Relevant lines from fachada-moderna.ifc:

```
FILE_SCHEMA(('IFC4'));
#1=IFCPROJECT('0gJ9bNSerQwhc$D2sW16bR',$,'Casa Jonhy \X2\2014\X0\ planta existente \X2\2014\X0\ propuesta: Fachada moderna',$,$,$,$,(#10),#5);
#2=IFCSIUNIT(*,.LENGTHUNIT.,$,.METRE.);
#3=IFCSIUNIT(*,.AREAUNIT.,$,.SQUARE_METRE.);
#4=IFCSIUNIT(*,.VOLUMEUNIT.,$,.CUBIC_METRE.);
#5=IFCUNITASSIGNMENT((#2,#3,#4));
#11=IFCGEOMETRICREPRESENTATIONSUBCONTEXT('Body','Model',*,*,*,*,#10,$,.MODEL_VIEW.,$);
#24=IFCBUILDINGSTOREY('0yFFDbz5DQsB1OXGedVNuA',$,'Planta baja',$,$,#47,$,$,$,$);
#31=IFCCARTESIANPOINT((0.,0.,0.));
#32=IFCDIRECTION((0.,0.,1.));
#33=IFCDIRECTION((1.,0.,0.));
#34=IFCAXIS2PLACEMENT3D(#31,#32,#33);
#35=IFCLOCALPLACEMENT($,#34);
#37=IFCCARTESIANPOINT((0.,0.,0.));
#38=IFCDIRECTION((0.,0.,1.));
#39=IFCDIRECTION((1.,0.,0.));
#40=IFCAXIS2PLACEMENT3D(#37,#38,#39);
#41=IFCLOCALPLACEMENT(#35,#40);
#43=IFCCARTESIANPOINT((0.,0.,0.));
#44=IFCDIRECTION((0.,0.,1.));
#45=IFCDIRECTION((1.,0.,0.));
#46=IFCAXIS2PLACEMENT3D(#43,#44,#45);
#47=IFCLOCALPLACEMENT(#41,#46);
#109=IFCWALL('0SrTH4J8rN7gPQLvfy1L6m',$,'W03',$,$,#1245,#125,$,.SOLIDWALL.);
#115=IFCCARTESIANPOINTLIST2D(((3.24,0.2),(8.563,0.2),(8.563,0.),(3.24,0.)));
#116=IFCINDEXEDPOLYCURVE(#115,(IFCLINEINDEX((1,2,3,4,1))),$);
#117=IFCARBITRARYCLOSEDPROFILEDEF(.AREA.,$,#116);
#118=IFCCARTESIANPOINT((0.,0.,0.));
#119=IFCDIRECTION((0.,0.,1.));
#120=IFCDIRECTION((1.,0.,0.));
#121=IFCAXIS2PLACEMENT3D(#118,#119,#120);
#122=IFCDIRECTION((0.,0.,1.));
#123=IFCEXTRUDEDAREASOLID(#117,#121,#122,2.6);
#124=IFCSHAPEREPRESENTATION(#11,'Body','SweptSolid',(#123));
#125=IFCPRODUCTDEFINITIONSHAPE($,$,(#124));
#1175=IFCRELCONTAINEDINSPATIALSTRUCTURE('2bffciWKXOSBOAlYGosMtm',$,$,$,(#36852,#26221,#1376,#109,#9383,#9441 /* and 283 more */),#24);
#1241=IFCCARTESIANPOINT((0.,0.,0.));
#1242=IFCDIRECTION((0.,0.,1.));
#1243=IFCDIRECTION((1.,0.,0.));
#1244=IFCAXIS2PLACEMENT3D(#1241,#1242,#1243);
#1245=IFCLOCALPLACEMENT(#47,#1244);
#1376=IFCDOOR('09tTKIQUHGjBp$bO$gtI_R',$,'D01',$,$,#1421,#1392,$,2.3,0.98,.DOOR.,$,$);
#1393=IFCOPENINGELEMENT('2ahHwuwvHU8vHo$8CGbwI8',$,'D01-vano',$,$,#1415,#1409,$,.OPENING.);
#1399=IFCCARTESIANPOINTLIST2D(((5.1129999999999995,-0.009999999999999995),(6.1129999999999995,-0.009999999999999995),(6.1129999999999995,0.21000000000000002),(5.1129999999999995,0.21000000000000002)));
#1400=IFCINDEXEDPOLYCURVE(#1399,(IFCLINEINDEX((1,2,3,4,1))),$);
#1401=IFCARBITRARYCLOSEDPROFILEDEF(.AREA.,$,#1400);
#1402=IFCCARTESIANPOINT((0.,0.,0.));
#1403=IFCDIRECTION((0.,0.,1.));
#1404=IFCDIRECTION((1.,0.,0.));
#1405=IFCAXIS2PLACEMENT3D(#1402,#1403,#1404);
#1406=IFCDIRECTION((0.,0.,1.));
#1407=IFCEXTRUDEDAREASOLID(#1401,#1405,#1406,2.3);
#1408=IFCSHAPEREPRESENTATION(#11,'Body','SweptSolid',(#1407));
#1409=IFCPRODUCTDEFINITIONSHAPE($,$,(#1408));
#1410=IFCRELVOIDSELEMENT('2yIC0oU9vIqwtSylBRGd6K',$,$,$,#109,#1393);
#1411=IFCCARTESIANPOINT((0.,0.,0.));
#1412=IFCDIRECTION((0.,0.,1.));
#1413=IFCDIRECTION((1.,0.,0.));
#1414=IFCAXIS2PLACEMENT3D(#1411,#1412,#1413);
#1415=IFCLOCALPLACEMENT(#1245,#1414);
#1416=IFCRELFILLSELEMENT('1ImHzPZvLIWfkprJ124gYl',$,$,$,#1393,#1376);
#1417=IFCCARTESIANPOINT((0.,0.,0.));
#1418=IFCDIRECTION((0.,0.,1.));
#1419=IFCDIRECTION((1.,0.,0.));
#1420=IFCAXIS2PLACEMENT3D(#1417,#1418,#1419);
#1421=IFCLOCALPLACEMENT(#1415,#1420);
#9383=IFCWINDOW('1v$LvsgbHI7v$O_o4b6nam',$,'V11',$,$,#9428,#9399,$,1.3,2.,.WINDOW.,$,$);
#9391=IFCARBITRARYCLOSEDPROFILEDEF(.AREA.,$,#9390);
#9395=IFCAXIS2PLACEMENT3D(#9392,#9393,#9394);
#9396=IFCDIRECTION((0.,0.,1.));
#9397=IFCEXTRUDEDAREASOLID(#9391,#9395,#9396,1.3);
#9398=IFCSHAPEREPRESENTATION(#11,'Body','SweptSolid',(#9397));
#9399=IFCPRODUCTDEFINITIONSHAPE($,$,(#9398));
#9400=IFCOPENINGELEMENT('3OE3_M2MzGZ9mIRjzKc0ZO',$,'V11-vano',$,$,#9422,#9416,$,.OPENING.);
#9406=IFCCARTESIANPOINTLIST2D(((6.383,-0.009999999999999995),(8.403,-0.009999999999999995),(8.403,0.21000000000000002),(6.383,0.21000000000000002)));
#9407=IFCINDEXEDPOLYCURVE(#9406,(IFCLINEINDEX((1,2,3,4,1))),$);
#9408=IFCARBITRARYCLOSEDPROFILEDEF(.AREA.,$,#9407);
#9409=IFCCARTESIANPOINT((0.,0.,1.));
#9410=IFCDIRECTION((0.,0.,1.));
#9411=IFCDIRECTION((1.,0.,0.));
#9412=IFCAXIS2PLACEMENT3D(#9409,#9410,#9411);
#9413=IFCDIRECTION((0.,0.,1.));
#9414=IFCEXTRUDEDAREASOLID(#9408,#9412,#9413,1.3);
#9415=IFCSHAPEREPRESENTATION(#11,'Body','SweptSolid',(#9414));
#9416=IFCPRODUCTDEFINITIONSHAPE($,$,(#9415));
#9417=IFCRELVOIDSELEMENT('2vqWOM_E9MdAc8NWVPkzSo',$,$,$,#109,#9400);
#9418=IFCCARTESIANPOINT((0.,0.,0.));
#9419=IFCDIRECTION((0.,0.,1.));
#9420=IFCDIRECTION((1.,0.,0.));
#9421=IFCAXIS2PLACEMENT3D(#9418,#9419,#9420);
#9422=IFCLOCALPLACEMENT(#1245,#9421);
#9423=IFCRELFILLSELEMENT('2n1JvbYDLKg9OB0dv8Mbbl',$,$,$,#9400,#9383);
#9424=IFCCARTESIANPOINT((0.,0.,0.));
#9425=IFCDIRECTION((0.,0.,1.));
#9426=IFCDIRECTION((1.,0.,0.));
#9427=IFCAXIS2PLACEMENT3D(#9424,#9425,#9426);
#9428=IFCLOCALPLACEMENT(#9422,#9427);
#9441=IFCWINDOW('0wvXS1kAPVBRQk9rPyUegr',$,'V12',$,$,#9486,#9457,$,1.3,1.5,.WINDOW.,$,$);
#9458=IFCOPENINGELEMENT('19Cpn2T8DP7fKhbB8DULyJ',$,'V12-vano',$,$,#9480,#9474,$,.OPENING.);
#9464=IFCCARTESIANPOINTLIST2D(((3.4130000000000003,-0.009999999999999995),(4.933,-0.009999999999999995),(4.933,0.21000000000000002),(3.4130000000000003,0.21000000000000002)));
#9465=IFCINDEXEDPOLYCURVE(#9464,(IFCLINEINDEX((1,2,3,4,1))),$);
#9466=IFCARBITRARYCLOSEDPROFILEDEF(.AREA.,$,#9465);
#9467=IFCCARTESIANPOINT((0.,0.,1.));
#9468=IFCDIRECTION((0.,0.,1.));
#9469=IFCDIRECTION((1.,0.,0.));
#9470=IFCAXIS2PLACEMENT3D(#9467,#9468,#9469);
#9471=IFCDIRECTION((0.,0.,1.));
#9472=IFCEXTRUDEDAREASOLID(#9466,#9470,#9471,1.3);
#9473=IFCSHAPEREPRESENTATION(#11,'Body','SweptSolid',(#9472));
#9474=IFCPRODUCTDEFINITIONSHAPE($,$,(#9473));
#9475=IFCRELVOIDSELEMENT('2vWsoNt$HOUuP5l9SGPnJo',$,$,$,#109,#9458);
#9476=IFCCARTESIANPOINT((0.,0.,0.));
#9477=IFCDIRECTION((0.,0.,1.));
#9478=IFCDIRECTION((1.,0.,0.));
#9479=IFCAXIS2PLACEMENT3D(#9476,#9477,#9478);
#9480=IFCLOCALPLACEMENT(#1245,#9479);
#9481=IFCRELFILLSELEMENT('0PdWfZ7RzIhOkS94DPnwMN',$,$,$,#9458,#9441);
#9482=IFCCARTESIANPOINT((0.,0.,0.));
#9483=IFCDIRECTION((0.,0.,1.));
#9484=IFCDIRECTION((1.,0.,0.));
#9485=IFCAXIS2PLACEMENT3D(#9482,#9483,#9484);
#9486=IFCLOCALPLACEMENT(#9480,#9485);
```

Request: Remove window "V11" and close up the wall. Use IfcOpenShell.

```python
import ifcopenshell
import ifcopenshell.api.feature
import ifcopenshell.api.root
import ifcopenshell.geom
import ifcopenshell.util.shape

model = ifcopenshell.open("fachada-moderna.ifc")
settings = ifcopenshell.geom.settings()


def volume(element):
    """Net volume in cubic metres, openings subtracted."""
    shape = ifcopenshell.geom.create_shape(settings, element)
    return ifcopenshell.util.shape.get_volume(shape.geometry)


window = model.by_id(9383)
opening = window.FillsVoids[0].RelatingOpeningElement
wall = opening.VoidsElements[0].RelatingBuildingElement
before = volume(wall)

ifcopenshell.api.root.remove_product(model, product=window)
ifcopenshell.api.feature.remove_feature(model, feature=opening)

after = volume(wall)

print(f"wall volume {before:.3f} -> {after:.3f} m3")

model.write("fachada-moderna_v2.ifc")
```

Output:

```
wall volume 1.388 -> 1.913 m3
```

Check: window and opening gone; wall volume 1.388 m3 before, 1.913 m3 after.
